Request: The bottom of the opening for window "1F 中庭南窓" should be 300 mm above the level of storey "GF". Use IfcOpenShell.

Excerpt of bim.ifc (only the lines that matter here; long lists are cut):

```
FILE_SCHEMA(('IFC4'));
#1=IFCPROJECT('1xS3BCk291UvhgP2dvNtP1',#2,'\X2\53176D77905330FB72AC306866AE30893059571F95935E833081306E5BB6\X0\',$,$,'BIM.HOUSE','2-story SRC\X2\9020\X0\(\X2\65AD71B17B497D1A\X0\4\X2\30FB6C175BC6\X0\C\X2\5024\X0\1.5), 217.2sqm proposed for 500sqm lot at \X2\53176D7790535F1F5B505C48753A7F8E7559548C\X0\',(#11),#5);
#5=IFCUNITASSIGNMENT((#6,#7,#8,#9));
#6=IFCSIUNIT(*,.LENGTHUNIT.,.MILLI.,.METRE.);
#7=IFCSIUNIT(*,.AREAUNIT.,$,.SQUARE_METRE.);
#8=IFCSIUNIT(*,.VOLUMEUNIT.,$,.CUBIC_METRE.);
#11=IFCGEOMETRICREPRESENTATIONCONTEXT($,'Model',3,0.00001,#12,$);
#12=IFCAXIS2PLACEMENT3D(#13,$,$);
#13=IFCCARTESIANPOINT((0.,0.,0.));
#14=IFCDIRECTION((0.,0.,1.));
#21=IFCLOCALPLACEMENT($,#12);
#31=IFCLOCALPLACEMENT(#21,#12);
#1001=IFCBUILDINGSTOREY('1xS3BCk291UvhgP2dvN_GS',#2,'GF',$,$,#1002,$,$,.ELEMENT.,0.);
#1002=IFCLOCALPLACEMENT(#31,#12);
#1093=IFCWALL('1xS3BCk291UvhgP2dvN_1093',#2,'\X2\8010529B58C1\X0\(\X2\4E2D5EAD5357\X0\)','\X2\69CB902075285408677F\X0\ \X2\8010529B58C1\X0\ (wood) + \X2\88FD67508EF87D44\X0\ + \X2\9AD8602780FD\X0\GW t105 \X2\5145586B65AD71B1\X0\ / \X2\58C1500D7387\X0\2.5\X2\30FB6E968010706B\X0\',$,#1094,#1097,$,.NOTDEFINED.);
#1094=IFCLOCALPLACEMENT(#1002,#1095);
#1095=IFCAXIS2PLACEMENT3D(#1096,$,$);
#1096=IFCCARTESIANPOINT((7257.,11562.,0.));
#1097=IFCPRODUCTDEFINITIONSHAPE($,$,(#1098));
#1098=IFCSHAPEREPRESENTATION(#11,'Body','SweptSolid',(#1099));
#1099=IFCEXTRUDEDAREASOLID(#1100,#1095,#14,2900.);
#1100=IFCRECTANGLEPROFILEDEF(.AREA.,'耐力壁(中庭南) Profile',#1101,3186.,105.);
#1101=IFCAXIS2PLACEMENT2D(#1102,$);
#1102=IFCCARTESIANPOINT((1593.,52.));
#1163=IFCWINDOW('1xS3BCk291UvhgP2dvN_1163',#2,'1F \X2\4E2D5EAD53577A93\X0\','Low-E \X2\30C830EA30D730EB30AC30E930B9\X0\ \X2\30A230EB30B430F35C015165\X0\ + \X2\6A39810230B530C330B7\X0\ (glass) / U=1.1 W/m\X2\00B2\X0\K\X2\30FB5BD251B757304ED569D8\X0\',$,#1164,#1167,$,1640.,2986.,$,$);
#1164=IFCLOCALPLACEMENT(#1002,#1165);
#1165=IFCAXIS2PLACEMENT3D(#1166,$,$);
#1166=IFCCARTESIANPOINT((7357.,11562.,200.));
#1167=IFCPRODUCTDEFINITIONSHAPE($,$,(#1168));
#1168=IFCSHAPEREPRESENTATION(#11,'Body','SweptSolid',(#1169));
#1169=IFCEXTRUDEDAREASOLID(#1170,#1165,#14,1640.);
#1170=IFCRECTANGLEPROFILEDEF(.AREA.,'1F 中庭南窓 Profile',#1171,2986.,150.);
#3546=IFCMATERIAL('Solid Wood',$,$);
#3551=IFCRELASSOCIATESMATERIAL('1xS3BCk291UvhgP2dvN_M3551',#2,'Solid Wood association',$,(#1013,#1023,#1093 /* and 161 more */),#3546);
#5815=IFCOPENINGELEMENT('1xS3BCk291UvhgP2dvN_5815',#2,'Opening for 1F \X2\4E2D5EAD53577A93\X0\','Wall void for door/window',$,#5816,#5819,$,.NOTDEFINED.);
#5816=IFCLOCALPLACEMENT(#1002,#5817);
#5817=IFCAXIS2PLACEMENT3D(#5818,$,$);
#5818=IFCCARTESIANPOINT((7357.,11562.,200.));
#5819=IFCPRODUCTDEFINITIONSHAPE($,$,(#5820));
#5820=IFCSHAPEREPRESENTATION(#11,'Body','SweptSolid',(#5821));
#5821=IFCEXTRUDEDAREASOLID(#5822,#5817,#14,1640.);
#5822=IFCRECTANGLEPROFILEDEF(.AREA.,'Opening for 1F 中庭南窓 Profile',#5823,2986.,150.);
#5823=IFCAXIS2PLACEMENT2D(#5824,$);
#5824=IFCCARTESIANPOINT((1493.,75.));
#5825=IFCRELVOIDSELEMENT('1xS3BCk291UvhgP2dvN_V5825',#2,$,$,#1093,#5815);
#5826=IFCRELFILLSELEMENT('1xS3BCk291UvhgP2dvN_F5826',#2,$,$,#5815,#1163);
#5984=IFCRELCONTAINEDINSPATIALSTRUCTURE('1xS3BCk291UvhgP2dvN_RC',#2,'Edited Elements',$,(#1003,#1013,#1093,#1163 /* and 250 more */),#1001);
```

```python
import numpy as np
import ifcopenshell
import ifcopenshell.api.geometry
import ifcopenshell.geom
import ifcopenshell.util.element
import ifcopenshell.util.placement
import ifcopenshell.util.shape
import ifcopenshell.util.unit

model = ifcopenshell.open("bim.ifc")
unit_scale = ifcopenshell.util.unit.calculate_unit_scale(model)

window = model.by_guid("1xS3BCk291UvhgP2dvN_1163")
opening = window.FillsVoids[0].RelatingOpeningElement
storey = ifcopenshell.util.element.get_container(window, ifc_class="IfcBuildingStorey")
level = ifcopenshell.util.placement.get_local_placement(storey.ObjectPlacement)[2, 3]

# The opening's origin need not be at the sill, so measure its lowest point.
shape = ifcopenshell.geom.create_shape(ifcopenshell.geom.settings(), opening)
bottom = ifcopenshell.util.shape.get_shape_bottom_elevation(shape, shape.geometry) / unit_scale
dz = level + 300.0 - bottom

shift = np.array([0.0, 0.0, dz])
# The window is not placed relative to its opening, so move both.
for product in (opening, window):
    matrix = ifcopenshell.util.placement.get_local_placement(product.ObjectPlacement)
    matrix[:3, 3] += shift
    ifcopenshell.api.geometry.edit_object_placement(model, product=product, matrix=matrix, is_si=False)

print(f"moved by {dz * unit_scale:+.3f} m")

model.write("bim_edited.ifc")
```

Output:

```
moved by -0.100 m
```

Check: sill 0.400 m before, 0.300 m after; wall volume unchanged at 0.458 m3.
